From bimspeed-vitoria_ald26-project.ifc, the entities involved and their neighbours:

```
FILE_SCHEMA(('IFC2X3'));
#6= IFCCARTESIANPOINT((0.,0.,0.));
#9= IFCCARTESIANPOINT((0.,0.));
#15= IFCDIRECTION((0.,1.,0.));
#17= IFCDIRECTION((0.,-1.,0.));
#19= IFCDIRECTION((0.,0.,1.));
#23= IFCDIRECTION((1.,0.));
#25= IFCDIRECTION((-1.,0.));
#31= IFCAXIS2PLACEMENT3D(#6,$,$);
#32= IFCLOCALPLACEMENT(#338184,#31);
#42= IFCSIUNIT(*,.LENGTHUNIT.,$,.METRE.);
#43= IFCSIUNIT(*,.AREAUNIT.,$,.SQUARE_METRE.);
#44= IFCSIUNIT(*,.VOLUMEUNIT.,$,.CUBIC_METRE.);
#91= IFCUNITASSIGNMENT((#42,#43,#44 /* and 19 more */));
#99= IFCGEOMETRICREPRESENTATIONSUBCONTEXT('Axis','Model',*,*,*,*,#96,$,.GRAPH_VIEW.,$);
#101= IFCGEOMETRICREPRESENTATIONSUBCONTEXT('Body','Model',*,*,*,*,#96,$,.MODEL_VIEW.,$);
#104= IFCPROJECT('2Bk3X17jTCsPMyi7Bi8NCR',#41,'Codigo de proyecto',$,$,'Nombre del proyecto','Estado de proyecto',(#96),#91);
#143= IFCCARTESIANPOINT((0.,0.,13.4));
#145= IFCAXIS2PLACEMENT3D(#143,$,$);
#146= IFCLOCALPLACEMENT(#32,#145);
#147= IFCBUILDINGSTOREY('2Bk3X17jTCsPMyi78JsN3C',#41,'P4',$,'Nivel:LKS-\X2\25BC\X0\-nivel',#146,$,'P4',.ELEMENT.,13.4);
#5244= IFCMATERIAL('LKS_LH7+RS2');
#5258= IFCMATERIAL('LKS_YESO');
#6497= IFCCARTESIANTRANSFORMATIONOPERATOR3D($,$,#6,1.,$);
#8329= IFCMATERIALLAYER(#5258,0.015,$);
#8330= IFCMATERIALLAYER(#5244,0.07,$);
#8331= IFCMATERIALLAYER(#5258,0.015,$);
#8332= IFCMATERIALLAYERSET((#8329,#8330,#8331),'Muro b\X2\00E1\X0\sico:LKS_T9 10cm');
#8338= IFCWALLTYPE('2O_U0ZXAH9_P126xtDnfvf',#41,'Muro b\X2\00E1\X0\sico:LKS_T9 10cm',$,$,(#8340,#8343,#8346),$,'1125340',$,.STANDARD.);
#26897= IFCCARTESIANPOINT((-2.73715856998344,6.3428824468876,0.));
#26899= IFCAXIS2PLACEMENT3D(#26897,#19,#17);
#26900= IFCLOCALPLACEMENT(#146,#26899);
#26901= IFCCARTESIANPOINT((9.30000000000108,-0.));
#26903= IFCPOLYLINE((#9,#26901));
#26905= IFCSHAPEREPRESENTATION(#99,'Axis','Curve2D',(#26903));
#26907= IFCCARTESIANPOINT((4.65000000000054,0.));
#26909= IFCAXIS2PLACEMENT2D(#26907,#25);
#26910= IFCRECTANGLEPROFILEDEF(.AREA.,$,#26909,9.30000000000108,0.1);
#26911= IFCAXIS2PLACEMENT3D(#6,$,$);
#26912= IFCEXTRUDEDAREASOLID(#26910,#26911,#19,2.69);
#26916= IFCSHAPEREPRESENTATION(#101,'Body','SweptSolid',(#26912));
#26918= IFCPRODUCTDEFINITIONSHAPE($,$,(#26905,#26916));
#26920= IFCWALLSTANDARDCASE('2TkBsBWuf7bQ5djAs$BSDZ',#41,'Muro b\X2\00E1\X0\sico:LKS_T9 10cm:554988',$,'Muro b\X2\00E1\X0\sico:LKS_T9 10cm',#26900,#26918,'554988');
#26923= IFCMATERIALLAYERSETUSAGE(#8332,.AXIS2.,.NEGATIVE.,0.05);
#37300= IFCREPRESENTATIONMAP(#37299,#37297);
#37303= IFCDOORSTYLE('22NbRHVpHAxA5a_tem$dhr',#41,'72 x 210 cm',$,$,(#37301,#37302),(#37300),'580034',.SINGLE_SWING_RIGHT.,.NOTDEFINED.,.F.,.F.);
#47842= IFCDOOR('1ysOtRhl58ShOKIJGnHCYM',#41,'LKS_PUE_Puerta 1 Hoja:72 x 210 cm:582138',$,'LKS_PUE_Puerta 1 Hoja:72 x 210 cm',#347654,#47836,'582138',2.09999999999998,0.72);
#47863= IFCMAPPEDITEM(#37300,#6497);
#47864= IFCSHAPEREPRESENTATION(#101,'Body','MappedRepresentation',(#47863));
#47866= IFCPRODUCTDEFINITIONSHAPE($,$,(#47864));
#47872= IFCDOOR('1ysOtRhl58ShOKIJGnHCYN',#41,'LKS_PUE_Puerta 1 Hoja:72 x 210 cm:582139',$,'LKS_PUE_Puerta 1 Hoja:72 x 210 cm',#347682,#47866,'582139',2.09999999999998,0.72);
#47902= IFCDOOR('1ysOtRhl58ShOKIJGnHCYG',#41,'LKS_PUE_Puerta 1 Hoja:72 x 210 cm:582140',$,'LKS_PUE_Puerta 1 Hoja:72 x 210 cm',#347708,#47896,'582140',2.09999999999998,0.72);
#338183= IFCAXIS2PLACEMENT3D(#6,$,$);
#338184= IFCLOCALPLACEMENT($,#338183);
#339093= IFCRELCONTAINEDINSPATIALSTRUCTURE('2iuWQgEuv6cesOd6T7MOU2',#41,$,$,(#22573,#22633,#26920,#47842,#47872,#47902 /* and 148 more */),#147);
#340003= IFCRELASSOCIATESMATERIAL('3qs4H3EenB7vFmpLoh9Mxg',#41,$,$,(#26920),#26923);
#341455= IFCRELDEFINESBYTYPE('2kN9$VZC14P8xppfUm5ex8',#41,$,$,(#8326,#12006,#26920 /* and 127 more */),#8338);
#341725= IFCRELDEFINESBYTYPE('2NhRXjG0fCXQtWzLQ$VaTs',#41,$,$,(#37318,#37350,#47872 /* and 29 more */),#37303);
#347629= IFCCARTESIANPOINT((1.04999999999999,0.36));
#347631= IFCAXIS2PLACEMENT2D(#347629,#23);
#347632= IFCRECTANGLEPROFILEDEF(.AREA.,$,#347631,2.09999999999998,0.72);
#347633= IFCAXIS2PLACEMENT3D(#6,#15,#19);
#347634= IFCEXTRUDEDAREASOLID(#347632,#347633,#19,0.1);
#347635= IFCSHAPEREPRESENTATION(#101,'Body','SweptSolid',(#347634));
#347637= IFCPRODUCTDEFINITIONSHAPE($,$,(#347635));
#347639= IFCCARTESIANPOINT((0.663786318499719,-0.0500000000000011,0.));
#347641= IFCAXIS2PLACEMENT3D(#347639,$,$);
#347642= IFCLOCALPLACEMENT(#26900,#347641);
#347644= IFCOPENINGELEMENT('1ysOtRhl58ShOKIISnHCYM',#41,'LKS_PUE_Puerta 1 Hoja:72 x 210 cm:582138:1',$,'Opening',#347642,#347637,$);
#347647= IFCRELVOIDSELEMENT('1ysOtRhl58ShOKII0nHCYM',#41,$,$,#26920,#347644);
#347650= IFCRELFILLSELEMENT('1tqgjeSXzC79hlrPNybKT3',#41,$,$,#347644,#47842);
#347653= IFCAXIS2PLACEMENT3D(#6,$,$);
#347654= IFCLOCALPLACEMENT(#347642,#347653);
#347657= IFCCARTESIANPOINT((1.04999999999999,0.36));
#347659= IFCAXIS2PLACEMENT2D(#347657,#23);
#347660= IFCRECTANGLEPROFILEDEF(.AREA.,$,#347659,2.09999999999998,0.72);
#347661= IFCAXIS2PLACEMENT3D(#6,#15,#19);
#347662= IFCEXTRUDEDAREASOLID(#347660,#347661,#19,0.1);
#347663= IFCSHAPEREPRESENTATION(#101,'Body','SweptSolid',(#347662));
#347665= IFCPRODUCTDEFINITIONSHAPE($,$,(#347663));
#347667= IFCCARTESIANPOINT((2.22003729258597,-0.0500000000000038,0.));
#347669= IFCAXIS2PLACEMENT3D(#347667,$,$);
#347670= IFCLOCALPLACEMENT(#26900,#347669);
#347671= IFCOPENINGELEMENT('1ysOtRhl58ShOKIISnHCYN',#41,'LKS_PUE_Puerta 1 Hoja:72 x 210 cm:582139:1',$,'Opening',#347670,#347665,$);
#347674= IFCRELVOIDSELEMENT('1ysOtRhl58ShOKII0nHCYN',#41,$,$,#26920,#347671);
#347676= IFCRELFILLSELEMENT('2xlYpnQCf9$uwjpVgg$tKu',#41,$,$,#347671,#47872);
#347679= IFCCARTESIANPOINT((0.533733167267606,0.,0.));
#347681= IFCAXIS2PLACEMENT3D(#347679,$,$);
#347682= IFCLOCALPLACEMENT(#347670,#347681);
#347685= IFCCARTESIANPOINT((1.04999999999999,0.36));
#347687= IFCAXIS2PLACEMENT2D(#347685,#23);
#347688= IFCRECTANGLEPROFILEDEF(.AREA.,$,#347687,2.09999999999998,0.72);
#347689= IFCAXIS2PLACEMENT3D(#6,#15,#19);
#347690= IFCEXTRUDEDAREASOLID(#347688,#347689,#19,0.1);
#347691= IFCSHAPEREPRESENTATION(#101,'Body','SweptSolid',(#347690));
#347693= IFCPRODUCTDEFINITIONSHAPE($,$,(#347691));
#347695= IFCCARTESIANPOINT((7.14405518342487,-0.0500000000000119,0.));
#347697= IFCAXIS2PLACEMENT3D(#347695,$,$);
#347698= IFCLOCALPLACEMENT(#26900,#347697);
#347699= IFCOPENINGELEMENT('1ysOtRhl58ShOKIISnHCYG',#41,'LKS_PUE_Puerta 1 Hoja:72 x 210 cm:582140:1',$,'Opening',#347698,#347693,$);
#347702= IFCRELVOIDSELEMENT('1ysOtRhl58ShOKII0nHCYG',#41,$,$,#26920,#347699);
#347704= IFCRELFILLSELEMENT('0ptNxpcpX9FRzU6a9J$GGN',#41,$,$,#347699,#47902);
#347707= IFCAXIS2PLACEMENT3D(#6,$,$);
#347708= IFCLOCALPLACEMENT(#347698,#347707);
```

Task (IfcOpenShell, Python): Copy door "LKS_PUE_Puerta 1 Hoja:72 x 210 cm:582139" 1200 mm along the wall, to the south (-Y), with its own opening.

```python
import ifcopenshell
import ifcopenshell.api.feature
import ifcopenshell.api.geometry
import ifcopenshell.api.root
import ifcopenshell.geom
import ifcopenshell.util.element
import ifcopenshell.util.placement
import ifcopenshell.util.shape
import ifcopenshell.util.unit

model = ifcopenshell.open("bimspeed-vitoria_ald26-project.ifc")
unit_scale = ifcopenshell.util.unit.calculate_unit_scale(model)
settings = ifcopenshell.geom.settings()


def volume(element):
    """Net volume in cubic metres, openings subtracted."""
    shape = ifcopenshell.geom.create_shape(settings, element)
    return ifcopenshell.util.shape.get_volume(shape.geometry)


def reuse_history(source, copy):
    """copy_class also copies each property set's owner history, people and application; keep the originals."""
    for rel in copy.IsDefinedBy:
        if rel.is_a("IfcRelDefinesByProperties") and (history := rel.RelatingPropertyDefinition.OwnerHistory):
            rel.RelatingPropertyDefinition.OwnerHistory = source.OwnerHistory
            ifcopenshell.util.element.remove_deep2(model, history)


door = model.by_guid("1ysOtRhl58ShOKIJGnHCYN")
opening = door.FillsVoids[0].RelatingOpeningElement
wall = opening.VoidsElements[0].RelatingBuildingElement
before = volume(wall)
shift = ifcopenshell.util.placement.get_local_placement(wall.ObjectPlacement)[:3, 0] * 1.2 / unit_scale

# copy_class copies the void relationship, type, container and properties, but no geometry.
new_opening = ifcopenshell.api.root.copy_class(model, product=opening)
new_opening.Representation = ifcopenshell.util.element.copy_deep(
    model, opening.Representation, exclude=["IfcGeometricRepresentationContext", "IfcRepresentationMap"]
)
new_opening.Name = "LKS_PUE_Puerta 1 Hoja:72 x 210 cm"
new_door = ifcopenshell.api.root.copy_class(model, product=door)
new_door.Representation = ifcopenshell.util.element.copy_deep(
    model, door.Representation, exclude=["IfcGeometricRepresentationContext", "IfcRepresentationMap"]
)
new_door.Name = "LKS_PUE_Puerta 1 Hoja:72 x 210 cm"
new_door.Tag = None
reuse_history(door, new_door)
fills = ifcopenshell.api.feature.add_filling(model, opening=new_opening, element=new_door)
fills.OwnerHistory = new_door.OwnerHistory  # required in IFC2X3

for old, new in ((opening, new_opening), (door, new_door)):
    matrix = ifcopenshell.util.placement.get_local_placement(old.ObjectPlacement)
    matrix[:3, 3] += shift
    ifcopenshell.api.geometry.edit_object_placement(model, product=new, matrix=matrix, is_si=False)

after = volume(wall)

print(f"wall volume {before:.3f} -> {after:.3f} m3")

model.write("bimspeed-vitoria_ald26-project_edited.ifc")
```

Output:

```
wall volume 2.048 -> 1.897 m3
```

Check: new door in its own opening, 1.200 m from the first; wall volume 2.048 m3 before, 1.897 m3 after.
